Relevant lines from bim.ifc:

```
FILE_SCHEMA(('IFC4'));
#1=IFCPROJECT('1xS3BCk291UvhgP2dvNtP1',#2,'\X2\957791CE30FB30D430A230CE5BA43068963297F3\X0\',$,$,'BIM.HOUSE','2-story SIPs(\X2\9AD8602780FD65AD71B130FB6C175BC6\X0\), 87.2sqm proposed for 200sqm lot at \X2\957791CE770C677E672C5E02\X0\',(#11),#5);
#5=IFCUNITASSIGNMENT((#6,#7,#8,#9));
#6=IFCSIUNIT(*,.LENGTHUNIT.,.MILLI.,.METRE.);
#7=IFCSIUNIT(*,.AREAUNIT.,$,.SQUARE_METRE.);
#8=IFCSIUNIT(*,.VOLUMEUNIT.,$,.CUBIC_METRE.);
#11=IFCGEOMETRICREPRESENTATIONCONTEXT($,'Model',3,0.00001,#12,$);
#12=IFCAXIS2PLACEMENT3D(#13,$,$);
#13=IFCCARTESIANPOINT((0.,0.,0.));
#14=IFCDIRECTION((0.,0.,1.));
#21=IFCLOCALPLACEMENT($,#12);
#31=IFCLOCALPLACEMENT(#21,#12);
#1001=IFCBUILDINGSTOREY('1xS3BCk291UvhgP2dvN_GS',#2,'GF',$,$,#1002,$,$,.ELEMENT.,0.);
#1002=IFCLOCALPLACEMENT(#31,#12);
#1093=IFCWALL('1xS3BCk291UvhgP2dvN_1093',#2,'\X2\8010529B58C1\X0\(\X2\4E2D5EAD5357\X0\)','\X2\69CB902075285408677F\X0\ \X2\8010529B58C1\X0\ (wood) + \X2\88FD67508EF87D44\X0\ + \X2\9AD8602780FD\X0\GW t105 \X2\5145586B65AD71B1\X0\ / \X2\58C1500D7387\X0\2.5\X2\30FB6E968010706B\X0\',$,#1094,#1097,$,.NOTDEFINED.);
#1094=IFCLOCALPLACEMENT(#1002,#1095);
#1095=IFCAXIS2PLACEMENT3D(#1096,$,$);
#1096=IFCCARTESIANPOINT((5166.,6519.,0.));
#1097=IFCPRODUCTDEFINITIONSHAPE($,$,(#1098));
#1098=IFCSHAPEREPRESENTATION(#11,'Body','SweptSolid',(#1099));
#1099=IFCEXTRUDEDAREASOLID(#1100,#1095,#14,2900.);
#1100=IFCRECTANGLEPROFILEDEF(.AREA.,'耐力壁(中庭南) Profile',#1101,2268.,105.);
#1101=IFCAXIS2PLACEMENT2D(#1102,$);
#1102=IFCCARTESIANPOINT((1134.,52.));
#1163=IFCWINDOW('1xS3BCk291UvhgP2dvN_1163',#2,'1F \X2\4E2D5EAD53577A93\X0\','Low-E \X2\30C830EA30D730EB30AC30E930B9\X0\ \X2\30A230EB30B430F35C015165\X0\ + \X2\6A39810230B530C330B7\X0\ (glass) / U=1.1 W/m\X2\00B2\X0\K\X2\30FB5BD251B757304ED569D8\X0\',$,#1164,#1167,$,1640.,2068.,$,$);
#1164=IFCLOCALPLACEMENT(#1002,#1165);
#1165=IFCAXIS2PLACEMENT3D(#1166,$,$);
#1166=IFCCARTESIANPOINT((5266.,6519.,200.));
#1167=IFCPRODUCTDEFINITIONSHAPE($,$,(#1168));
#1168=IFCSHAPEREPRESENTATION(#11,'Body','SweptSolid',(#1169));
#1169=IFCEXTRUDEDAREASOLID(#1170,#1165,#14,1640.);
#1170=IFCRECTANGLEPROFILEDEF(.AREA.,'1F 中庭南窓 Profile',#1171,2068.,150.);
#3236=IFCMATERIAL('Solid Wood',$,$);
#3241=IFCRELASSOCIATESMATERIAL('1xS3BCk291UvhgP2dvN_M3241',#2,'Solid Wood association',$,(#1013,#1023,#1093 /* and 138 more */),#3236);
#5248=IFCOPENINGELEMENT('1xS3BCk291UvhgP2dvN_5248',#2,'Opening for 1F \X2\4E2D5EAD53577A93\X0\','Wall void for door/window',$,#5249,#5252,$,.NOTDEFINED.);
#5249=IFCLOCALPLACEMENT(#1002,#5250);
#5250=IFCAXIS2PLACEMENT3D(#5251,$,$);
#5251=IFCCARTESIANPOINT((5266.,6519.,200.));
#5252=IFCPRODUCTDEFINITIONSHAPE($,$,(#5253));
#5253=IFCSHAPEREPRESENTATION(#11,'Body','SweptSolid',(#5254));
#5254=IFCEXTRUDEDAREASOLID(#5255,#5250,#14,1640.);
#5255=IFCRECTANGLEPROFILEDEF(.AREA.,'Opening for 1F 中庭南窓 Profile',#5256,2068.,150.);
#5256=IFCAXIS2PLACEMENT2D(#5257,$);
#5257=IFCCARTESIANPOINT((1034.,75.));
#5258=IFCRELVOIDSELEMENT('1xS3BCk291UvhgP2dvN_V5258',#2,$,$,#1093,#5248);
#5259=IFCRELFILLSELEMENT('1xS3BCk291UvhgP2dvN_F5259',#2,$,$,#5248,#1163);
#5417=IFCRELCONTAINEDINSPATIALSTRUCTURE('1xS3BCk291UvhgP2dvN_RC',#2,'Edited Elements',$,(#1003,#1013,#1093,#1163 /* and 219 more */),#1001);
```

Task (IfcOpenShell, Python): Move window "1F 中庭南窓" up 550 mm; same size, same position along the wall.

```python
import numpy as np
import ifcopenshell
import ifcopenshell.api.geometry
import ifcopenshell.util.placement
import ifcopenshell.util.unit

model = ifcopenshell.open("bim.ifc")
unit_scale = ifcopenshell.util.unit.calculate_unit_scale(model)

window = model.by_id(1163)
opening = window.FillsVoids[0].RelatingOpeningElement
dz = 0.55 / unit_scale

shift = np.array([0.0, 0.0, dz])
# The window is not placed relative to its opening, so move both.
for product in (opening, window):
    matrix = ifcopenshell.util.placement.get_local_placement(product.ObjectPlacement)
    matrix[:3, 3] += shift
    ifcopenshell.api.geometry.edit_object_placement(model, product=product, matrix=matrix, is_si=False)

print(f"moved by {dz * unit_scale:+.3f} m")

model.write("bim_v2.ifc")
```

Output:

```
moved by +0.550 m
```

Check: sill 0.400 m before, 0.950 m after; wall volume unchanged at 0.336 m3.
